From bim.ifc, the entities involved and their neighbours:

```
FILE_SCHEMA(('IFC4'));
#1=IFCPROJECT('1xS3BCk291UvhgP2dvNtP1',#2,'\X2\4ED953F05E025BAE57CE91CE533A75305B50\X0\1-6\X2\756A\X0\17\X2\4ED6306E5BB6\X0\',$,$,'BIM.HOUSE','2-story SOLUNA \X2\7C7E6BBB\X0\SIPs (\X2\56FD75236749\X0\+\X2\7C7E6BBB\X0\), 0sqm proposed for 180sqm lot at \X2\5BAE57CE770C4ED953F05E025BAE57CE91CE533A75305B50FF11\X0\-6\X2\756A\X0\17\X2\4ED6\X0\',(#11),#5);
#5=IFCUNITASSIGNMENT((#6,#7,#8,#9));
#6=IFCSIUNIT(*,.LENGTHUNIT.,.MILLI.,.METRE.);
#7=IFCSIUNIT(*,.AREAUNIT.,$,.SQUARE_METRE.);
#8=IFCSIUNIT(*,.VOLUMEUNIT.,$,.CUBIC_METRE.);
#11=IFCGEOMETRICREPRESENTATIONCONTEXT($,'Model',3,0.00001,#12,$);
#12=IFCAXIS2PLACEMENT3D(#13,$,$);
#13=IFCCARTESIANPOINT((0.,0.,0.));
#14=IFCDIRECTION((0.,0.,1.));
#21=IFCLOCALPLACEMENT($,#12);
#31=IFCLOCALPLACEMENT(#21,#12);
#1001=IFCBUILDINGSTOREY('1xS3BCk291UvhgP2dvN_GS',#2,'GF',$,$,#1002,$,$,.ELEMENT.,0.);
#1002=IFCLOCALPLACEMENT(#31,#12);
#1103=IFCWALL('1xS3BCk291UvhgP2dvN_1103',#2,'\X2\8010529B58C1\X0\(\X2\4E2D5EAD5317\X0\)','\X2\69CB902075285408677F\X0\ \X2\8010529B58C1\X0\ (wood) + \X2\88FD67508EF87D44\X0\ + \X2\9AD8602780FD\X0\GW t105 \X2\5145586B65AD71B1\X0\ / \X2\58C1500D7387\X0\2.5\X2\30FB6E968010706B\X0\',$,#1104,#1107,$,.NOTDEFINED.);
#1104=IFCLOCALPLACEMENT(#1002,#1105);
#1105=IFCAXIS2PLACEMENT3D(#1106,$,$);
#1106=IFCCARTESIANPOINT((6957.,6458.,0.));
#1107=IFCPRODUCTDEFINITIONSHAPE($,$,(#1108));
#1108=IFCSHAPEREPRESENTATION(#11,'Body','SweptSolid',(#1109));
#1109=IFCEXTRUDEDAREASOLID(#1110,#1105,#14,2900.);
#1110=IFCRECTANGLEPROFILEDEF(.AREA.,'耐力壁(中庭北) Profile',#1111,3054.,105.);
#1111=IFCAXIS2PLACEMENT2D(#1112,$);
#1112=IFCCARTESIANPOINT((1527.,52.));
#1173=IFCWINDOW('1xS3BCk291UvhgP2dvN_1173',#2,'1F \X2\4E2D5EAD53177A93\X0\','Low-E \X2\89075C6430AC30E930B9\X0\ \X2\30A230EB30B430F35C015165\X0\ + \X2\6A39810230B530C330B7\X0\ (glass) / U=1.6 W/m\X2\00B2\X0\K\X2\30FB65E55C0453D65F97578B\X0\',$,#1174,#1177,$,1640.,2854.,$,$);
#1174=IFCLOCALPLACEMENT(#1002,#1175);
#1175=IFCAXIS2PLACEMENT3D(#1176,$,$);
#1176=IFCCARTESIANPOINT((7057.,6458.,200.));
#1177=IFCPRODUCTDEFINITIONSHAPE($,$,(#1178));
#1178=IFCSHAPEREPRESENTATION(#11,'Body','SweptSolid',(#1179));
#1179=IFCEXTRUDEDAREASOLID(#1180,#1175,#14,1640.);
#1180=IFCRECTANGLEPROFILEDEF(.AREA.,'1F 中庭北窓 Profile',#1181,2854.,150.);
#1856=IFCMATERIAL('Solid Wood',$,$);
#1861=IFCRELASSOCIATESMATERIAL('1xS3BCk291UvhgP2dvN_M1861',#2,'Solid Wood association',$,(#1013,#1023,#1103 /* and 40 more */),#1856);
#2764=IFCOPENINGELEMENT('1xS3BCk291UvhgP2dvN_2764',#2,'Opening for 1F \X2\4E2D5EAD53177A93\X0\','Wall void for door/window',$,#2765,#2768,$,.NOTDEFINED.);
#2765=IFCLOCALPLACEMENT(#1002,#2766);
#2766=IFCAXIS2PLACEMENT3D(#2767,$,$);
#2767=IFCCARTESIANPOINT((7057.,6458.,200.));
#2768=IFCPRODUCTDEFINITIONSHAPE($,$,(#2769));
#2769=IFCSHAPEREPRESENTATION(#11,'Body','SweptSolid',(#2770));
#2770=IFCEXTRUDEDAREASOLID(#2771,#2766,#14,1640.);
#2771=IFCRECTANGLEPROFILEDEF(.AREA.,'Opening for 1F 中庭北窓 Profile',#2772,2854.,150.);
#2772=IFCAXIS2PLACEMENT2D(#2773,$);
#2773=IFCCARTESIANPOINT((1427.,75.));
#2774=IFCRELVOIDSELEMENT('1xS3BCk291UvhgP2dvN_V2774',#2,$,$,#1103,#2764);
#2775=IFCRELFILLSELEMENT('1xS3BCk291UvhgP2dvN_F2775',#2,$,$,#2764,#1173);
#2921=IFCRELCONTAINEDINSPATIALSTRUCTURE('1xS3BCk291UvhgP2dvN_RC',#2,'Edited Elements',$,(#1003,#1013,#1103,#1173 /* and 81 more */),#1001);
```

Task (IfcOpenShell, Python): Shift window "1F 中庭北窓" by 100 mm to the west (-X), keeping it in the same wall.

```python
import ifcopenshell
import ifcopenshell.api.geometry
import ifcopenshell.util.placement
import ifcopenshell.util.unit

model = ifcopenshell.open("bim.ifc")
unit_scale = ifcopenshell.util.unit.calculate_unit_scale(model)

window = model.by_id(1173)
opening = window.FillsVoids[0].RelatingOpeningElement
wall = opening.VoidsElements[0].RelatingBuildingElement

wall_matrix = ifcopenshell.util.placement.get_local_placement(wall.ObjectPlacement)
shift = wall_matrix[:3, 0] * -0.1 / unit_scale
before = ifcopenshell.util.placement.get_local_placement(window.ObjectPlacement)[:3, 3].copy()

# The window is not placed relative to its opening, so move both.
for product in (opening, window):
    matrix = ifcopenshell.util.placement.get_local_placement(product.ObjectPlacement)
    matrix[:3, 3] += shift
    ifcopenshell.api.geometry.edit_object_placement(model, product=product, matrix=matrix, is_si=False)

after = ifcopenshell.util.placement.get_local_placement(window.ObjectPlacement)[:3, 3]
print("window moved by", (after - before).round(3) + 0.0)

model.write("bim_v2.ifc")
```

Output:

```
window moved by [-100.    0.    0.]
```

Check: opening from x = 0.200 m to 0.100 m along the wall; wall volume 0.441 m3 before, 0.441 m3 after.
